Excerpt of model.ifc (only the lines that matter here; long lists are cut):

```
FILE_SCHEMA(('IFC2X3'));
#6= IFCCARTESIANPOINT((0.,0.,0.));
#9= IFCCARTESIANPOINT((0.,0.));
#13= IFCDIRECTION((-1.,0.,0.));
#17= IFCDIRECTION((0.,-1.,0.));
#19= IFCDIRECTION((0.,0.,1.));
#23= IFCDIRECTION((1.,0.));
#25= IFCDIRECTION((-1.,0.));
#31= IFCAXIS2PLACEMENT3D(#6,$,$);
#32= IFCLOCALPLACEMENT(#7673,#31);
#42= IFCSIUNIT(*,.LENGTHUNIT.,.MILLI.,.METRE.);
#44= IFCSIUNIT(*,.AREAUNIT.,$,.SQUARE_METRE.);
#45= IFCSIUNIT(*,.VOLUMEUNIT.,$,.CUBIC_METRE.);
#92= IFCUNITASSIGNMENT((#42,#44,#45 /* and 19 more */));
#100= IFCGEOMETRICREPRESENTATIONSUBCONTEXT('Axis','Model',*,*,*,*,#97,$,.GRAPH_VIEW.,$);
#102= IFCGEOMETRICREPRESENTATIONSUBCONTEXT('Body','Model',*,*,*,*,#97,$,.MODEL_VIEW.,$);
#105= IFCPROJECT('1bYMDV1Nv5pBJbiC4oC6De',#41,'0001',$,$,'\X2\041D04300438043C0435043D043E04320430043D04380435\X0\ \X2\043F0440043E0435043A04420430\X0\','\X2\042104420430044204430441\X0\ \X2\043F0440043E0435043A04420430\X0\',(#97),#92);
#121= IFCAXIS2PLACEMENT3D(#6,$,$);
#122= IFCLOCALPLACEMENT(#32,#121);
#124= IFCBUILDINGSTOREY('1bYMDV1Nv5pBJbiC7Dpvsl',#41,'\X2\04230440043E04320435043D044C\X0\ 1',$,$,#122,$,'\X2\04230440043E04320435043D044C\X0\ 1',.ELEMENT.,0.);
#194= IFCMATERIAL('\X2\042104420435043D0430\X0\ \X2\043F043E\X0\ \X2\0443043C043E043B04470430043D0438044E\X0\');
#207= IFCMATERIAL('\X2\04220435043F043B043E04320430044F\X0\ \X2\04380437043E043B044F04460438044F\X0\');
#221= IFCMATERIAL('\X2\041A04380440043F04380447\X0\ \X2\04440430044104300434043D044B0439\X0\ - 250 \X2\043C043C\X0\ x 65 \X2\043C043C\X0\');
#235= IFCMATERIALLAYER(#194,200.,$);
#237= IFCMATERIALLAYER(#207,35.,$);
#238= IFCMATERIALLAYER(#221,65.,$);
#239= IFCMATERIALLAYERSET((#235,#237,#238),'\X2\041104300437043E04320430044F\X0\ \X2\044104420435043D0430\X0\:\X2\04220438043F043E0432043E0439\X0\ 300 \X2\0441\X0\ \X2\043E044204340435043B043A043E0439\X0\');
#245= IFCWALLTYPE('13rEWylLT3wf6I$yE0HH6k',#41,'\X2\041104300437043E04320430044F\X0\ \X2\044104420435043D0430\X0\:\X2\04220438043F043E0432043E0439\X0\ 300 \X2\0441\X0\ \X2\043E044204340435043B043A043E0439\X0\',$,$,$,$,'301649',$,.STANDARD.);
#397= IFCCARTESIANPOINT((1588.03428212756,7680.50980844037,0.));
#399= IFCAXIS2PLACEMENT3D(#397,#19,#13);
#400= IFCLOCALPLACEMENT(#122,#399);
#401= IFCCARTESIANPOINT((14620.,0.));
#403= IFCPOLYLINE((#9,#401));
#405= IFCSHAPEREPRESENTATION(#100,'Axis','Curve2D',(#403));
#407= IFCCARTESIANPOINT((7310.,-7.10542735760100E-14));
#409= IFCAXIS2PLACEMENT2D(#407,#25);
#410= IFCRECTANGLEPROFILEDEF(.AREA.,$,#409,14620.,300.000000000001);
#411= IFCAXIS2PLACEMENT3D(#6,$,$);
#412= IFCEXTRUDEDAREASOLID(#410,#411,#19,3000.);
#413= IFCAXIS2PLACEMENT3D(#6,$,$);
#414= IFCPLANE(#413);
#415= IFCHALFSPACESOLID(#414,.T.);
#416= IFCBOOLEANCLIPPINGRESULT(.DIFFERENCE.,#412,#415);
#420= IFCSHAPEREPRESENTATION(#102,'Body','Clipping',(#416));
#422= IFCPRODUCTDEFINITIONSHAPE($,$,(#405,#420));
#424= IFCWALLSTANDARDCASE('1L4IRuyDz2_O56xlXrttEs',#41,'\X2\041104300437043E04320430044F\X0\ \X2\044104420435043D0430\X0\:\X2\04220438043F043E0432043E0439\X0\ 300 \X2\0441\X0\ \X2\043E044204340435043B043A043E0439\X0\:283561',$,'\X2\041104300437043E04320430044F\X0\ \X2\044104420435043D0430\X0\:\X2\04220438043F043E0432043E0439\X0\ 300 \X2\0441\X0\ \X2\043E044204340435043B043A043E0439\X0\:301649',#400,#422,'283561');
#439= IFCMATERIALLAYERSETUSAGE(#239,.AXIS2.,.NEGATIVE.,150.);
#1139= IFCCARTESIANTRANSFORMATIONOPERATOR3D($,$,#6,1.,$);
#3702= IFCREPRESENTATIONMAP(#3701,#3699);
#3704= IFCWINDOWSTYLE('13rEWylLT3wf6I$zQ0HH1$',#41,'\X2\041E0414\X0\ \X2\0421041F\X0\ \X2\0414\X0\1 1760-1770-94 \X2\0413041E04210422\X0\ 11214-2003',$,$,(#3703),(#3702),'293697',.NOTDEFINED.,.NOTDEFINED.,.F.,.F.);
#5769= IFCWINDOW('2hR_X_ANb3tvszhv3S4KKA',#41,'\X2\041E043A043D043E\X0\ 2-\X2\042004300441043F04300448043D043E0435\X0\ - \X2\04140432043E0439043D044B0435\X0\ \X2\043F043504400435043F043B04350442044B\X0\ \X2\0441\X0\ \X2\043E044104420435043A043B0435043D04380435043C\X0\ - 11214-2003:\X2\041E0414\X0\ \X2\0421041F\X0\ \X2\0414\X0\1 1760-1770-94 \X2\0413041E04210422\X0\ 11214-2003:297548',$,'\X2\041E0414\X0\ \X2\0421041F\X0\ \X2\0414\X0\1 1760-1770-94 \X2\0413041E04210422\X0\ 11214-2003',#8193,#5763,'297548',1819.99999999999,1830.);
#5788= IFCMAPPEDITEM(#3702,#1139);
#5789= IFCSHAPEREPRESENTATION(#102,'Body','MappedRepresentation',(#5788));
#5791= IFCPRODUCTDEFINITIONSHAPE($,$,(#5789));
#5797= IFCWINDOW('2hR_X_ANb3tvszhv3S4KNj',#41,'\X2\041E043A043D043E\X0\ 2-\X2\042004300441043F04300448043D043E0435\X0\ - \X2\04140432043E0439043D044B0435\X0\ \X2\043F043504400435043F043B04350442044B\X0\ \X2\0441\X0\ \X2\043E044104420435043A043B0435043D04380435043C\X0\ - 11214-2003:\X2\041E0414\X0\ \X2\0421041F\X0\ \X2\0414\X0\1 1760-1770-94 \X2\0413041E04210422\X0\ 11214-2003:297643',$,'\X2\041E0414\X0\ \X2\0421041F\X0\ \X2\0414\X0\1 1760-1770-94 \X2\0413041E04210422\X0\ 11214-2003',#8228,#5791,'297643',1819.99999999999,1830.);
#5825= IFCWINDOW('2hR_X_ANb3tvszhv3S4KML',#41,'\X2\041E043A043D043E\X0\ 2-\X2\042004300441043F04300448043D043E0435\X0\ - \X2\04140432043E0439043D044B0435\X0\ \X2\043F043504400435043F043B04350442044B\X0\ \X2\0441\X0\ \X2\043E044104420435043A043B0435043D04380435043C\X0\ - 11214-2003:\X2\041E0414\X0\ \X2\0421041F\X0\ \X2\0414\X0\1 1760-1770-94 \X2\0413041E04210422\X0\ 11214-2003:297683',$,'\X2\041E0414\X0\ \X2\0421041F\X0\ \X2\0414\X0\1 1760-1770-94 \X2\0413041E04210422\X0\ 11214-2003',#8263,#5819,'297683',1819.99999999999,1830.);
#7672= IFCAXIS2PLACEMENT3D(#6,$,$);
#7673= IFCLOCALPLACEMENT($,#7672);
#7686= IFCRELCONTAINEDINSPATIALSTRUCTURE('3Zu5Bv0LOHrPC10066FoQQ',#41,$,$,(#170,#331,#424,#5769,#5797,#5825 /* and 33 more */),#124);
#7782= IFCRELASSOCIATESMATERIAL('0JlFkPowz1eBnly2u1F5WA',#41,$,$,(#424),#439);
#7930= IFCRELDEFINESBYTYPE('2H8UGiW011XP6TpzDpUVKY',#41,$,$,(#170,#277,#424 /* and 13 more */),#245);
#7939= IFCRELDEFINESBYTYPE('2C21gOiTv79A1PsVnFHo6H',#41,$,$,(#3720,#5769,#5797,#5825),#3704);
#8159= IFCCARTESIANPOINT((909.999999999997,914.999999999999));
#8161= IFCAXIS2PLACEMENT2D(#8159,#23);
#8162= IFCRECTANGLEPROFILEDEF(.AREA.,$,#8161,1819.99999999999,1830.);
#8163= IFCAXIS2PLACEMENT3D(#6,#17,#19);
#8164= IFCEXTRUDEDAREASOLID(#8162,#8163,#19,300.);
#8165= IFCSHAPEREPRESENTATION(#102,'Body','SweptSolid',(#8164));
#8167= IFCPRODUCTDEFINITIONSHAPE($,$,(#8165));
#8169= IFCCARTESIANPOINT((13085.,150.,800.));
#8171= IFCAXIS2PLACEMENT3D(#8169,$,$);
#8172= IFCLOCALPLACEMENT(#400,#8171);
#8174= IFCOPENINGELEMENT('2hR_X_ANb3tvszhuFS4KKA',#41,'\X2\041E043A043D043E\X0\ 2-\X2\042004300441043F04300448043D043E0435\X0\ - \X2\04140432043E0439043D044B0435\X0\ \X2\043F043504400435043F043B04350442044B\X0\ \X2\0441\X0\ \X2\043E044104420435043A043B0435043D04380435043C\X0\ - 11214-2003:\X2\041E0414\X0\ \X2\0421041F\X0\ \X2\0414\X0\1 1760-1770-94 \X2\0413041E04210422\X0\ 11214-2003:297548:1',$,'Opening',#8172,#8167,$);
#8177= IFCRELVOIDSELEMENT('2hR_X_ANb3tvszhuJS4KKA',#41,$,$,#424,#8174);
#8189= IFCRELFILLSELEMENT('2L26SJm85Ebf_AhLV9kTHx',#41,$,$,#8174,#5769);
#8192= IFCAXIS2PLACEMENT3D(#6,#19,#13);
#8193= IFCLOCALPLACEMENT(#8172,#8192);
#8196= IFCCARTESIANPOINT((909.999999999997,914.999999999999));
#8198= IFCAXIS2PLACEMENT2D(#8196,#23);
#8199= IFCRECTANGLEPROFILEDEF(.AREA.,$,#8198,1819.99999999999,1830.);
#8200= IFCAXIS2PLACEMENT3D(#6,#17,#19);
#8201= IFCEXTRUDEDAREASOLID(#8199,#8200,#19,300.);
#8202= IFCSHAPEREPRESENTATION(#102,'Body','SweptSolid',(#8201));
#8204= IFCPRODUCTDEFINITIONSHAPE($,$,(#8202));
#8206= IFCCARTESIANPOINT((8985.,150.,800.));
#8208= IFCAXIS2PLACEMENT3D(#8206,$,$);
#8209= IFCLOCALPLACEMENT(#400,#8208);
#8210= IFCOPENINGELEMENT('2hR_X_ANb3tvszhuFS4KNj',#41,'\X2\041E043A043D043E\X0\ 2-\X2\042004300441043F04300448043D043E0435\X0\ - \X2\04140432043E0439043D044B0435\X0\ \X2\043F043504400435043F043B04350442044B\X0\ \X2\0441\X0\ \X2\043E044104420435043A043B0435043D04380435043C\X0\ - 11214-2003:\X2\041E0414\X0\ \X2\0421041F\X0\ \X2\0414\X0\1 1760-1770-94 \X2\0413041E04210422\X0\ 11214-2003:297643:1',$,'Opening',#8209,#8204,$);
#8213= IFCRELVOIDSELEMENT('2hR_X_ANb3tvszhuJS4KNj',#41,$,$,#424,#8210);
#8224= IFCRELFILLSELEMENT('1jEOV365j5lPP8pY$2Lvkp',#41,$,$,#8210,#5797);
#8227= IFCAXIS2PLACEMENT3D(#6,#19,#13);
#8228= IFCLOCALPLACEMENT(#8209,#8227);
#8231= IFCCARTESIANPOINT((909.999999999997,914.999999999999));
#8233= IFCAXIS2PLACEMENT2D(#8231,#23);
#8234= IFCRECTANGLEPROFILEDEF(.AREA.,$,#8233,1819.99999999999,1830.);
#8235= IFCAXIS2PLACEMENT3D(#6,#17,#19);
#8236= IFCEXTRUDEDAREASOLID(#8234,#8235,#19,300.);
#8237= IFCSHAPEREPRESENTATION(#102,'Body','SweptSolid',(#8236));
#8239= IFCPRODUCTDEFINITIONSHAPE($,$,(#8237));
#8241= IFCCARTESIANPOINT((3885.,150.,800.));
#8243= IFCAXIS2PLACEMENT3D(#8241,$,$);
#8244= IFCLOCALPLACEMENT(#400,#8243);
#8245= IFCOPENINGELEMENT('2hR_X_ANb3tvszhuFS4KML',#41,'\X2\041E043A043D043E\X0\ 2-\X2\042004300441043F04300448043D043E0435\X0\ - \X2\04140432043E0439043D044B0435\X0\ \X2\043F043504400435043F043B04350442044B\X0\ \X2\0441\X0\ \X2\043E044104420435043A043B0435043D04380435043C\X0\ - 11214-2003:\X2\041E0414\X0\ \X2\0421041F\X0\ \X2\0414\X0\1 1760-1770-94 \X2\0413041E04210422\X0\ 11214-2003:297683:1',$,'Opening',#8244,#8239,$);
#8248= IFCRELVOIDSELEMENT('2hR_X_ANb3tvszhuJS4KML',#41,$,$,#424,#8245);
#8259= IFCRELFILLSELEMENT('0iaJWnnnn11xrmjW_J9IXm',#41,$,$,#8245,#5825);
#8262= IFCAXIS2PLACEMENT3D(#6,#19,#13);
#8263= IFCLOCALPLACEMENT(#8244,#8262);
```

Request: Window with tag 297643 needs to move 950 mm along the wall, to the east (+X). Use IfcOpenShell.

```python
import ifcopenshell
import ifcopenshell.api.geometry
import ifcopenshell.util.placement
import ifcopenshell.util.unit

model = ifcopenshell.open("model.ifc")
unit_scale = ifcopenshell.util.unit.calculate_unit_scale(model)

window = model.by_id(5797)
opening = window.FillsVoids[0].RelatingOpeningElement
wall = opening.VoidsElements[0].RelatingBuildingElement

wall_matrix = ifcopenshell.util.placement.get_local_placement(wall.ObjectPlacement)
shift = wall_matrix[:3, 0] * -0.95 / unit_scale
before = ifcopenshell.util.placement.get_local_placement(window.ObjectPlacement)[:3, 3].copy()

# The window is placed relative to its opening, so it follows when the opening moves.
matrix = ifcopenshell.util.placement.get_local_placement(opening.ObjectPlacement)
matrix[:3, 3] += shift
ifcopenshell.api.geometry.edit_object_placement(
    model, product=opening, matrix=matrix, is_si=False, should_transform_children=True
)

after = ifcopenshell.util.placement.get_local_placement(window.ObjectPlacement)[:3, 3]
print("window moved by", (after - before).round(3) + 0.0)

model.write("model_edited.ifc")
```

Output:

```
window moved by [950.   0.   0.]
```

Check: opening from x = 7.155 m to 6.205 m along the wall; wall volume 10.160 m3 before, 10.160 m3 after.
